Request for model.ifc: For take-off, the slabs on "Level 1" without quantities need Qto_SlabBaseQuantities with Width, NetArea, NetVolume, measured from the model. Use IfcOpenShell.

First a look at what the model holds.

```python
import ifcopenshell
import ifcopenshell.util.element
import ifcopenshell.util.unit

model = ifcopenshell.open("model.ifc")
print(model.schema)
for unit_type in ("LENGTHUNIT", "AREAUNIT", "VOLUMEUNIT"):
    print(unit_type, ifcopenshell.util.unit.calculate_unit_scale(model, unit_type))
storey = next(s for s in model.by_type("IfcBuildingStorey") if s.Name == "Level 1")
slabs = [e for e in ifcopenshell.util.element.get_decomposition(storey) if e.is_a("IfcSlab")]
for e in sorted(slabs, key=lambda e: e.id()):
    print(e.id(), e.is_a(), e.Name, list(ifcopenshell.util.element.get_psets(e, qtos_only=True)), sep=" | ")
```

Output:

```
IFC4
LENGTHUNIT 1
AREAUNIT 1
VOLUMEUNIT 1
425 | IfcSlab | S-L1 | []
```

```python
import ifcopenshell
import ifcopenshell.api.pset
import ifcopenshell.geom
import ifcopenshell.util.element
import ifcopenshell.util.shape
import ifcopenshell.util.unit

model = ifcopenshell.open("model.ifc")
unit_scale = ifcopenshell.util.unit.calculate_unit_scale(model)
area_scale = ifcopenshell.util.unit.calculate_unit_scale(model, "AREAUNIT")
volume_scale = ifcopenshell.util.unit.calculate_unit_scale(model, "VOLUMEUNIT")
settings = ifcopenshell.geom.settings()

storey = next(s for s in model.by_type("IfcBuildingStorey") if s.Name == "Level 1")
slabs = [e for e in ifcopenshell.util.element.get_decomposition(storey) if e.is_a("IfcSlab")]

for e in sorted(slabs, key=lambda e: e.id()):
    if ifcopenshell.util.element.get_psets(e, qtos_only=True, should_inherit=False):
        continue
    # Geometry comes back in metres, in the element's own axes.
    shape = ifcopenshell.geom.create_shape(settings, e)
    values = {
        "Width": ifcopenshell.util.shape.get_z(shape.geometry) / unit_scale,
        "NetArea": ifcopenshell.util.shape.get_footprint_area(shape.geometry) / area_scale,
        "NetVolume": ifcopenshell.util.shape.get_volume(shape.geometry) / volume_scale,
    }
    qto = ifcopenshell.api.pset.add_qto(model, product=e, name="Qto_SlabBaseQuantities")
    ifcopenshell.api.pset.edit_qto(model, qto=qto, properties=values)
    print(e.id(), {k: round(v, 3) for k, v in values.items()})

model.write("model_rev.ifc")
```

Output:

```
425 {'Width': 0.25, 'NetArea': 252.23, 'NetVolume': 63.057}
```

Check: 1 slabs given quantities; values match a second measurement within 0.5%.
